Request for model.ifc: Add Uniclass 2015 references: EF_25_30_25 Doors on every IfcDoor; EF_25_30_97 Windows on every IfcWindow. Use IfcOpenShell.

First a look at what the model holds.

```python
import ifcopenshell

model = ifcopenshell.open("model.ifc")
print(model.schema)
print("classifications:", [c.Name for c in model.by_type("IfcClassification")])
for ifc_class in ("IfcDoor", "IfcRoof", "IfcStair", "IfcWall", "IfcWindow"):
    print(ifc_class, len(model.by_type(ifc_class)))
```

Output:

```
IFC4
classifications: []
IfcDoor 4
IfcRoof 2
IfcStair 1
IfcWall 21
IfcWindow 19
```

```python
import ifcopenshell
import ifcopenshell.api.classification

model = ifcopenshell.open("model.ifc")

system = ifcopenshell.api.classification.add_classification(model, classification="Uniclass 2015")

codes = {
    "IfcDoor": ("EF_25_30_25", "Doors"),
    "IfcWindow": ("EF_25_30_97", "Windows"),
}
for ifc_class, (code, name) in codes.items():
    products = model.by_type(ifc_class)
    ifcopenshell.api.classification.add_reference(
        model, products=products, classification=system, identification=code, name=name
    )
    print(code, len(products))

model.write("model_edited.ifc")
```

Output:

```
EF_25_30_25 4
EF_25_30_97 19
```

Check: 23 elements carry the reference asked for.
